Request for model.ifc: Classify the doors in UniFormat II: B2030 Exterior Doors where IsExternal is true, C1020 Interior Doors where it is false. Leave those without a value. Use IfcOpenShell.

First a look at what the model holds.

```python
import ifcopenshell
import ifcopenshell.util.element

model = ifcopenshell.open("model.ifc")
print(model.schema)
print("classifications:", [c.Name for c in model.by_type("IfcClassification")])
values = [ifcopenshell.util.element.get_pset(e, "Pset_DoorCommon", "IsExternal") for e in model.by_type("IfcDoor")]
for value in (True, False, None):
    print("IsExternal", value, values.count(value))
```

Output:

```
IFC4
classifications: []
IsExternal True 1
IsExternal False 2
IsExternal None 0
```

```python
import ifcopenshell
import ifcopenshell.api.classification
import ifcopenshell.util.element

model = ifcopenshell.open("model.ifc")

system = ifcopenshell.api.classification.add_classification(model, classification="UniFormat II")

doors = model.by_type("IfcDoor")
external = {e: ifcopenshell.util.element.get_pset(e, "Pset_DoorCommon", "IsExternal") for e in doors}
for flag, code, name in ((True, "B2030", "Exterior Doors"), (False, "C1020", "Interior Doors")):
    products = [e for e in doors if external[e] is flag]
    ifcopenshell.api.classification.add_reference(
        model, products=products, classification=system, identification=code, name=name
    )
    print(code, len(products))

model.write("model_edited.ifc")
```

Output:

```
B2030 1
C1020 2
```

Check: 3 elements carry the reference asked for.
